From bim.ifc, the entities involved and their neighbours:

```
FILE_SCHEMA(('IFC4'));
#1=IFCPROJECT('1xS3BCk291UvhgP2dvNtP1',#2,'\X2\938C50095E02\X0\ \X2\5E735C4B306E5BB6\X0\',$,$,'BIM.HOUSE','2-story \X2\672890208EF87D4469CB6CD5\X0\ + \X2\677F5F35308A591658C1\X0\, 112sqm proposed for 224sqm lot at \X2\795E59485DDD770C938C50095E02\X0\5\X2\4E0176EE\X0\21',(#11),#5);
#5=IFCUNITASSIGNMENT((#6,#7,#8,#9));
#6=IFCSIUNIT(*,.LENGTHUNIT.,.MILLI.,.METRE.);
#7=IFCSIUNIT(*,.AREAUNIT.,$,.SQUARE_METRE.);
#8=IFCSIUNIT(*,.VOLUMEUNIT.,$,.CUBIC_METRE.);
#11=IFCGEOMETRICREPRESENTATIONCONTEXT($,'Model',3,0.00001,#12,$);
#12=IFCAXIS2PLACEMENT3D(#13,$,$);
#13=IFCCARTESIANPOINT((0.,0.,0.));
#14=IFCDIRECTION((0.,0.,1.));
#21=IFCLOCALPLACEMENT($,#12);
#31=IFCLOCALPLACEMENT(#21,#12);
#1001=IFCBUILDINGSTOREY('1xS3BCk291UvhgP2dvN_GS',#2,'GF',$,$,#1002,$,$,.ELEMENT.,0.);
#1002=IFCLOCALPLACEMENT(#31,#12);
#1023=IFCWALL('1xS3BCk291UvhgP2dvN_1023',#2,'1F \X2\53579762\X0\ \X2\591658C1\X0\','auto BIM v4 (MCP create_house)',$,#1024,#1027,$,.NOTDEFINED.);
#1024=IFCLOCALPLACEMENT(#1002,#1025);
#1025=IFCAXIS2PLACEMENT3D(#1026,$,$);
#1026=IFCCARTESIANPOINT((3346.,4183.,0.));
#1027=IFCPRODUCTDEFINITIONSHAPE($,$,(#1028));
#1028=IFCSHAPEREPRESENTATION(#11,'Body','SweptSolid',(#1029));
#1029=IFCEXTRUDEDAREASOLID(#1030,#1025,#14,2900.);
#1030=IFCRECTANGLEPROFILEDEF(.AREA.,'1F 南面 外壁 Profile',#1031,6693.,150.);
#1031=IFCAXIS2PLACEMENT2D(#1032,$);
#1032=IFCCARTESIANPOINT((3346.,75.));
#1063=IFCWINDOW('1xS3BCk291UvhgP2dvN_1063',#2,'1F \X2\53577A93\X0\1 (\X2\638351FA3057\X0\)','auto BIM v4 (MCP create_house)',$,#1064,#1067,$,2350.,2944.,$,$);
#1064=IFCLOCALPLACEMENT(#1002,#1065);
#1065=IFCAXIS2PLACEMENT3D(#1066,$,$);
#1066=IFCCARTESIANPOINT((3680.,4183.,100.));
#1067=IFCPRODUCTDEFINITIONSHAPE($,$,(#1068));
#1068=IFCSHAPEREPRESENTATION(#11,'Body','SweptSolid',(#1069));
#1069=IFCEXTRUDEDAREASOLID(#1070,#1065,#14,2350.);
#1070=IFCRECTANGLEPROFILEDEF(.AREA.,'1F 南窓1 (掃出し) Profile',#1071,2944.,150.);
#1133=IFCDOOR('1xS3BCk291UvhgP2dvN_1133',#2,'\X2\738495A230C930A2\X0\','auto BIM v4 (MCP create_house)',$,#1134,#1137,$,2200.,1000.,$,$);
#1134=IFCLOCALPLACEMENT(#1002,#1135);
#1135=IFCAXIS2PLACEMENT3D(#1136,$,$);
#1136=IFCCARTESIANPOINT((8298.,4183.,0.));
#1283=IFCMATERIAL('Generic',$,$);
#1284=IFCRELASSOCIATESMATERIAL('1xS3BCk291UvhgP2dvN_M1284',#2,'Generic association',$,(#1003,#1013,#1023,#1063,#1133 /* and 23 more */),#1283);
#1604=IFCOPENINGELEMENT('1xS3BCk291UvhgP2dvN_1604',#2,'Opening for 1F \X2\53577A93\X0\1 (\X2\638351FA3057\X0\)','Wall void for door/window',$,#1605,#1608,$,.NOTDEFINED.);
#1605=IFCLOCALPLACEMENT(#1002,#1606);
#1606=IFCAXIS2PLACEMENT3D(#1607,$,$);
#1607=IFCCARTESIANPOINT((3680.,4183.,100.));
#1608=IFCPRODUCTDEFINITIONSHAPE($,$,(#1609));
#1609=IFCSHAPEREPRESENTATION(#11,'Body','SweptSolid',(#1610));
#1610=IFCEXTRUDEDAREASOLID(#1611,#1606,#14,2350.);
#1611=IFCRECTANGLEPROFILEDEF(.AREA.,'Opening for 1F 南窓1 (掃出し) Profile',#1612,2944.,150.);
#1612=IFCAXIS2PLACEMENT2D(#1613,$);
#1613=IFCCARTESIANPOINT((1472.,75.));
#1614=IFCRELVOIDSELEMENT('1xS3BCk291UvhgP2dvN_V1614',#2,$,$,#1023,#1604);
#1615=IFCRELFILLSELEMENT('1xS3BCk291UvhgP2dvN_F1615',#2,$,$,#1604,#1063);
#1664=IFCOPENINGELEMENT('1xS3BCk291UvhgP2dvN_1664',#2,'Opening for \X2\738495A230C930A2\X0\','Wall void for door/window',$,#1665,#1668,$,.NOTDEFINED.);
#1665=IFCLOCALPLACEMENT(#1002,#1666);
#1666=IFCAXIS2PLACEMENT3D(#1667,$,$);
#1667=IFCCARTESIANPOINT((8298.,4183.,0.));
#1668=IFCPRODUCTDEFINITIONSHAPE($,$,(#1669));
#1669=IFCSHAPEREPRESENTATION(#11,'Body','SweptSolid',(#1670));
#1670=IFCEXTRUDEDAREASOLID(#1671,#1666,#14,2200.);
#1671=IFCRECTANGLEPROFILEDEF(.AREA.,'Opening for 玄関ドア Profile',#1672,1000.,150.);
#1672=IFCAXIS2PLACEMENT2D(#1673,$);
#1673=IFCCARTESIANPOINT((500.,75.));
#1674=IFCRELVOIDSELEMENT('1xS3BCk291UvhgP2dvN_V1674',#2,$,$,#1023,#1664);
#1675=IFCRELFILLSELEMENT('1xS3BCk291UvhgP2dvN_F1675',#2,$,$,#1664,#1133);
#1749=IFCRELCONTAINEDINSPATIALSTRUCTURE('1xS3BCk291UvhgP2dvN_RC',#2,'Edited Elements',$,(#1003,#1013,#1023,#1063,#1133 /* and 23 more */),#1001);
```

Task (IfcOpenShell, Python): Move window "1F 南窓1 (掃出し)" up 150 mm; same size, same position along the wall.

```python
import numpy as np
import ifcopenshell
import ifcopenshell.api.geometry
import ifcopenshell.util.placement
import ifcopenshell.util.unit

model = ifcopenshell.open("bim.ifc")
unit_scale = ifcopenshell.util.unit.calculate_unit_scale(model)

window = model.by_guid("1xS3BCk291UvhgP2dvN_1063")
opening = window.FillsVoids[0].RelatingOpeningElement
dz = 150.0

shift = np.array([0.0, 0.0, dz])
# The window is not placed relative to its opening, so move both.
for product in (opening, window):
    matrix = ifcopenshell.util.placement.get_local_placement(product.ObjectPlacement)
    matrix[:3, 3] += shift
    ifcopenshell.api.geometry.edit_object_placement(model, product=product, matrix=matrix, is_si=False)

print(f"moved by {dz * unit_scale:+.3f} m")

model.write("bim_updated.ifc")
```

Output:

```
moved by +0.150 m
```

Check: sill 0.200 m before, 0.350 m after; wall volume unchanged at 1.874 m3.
